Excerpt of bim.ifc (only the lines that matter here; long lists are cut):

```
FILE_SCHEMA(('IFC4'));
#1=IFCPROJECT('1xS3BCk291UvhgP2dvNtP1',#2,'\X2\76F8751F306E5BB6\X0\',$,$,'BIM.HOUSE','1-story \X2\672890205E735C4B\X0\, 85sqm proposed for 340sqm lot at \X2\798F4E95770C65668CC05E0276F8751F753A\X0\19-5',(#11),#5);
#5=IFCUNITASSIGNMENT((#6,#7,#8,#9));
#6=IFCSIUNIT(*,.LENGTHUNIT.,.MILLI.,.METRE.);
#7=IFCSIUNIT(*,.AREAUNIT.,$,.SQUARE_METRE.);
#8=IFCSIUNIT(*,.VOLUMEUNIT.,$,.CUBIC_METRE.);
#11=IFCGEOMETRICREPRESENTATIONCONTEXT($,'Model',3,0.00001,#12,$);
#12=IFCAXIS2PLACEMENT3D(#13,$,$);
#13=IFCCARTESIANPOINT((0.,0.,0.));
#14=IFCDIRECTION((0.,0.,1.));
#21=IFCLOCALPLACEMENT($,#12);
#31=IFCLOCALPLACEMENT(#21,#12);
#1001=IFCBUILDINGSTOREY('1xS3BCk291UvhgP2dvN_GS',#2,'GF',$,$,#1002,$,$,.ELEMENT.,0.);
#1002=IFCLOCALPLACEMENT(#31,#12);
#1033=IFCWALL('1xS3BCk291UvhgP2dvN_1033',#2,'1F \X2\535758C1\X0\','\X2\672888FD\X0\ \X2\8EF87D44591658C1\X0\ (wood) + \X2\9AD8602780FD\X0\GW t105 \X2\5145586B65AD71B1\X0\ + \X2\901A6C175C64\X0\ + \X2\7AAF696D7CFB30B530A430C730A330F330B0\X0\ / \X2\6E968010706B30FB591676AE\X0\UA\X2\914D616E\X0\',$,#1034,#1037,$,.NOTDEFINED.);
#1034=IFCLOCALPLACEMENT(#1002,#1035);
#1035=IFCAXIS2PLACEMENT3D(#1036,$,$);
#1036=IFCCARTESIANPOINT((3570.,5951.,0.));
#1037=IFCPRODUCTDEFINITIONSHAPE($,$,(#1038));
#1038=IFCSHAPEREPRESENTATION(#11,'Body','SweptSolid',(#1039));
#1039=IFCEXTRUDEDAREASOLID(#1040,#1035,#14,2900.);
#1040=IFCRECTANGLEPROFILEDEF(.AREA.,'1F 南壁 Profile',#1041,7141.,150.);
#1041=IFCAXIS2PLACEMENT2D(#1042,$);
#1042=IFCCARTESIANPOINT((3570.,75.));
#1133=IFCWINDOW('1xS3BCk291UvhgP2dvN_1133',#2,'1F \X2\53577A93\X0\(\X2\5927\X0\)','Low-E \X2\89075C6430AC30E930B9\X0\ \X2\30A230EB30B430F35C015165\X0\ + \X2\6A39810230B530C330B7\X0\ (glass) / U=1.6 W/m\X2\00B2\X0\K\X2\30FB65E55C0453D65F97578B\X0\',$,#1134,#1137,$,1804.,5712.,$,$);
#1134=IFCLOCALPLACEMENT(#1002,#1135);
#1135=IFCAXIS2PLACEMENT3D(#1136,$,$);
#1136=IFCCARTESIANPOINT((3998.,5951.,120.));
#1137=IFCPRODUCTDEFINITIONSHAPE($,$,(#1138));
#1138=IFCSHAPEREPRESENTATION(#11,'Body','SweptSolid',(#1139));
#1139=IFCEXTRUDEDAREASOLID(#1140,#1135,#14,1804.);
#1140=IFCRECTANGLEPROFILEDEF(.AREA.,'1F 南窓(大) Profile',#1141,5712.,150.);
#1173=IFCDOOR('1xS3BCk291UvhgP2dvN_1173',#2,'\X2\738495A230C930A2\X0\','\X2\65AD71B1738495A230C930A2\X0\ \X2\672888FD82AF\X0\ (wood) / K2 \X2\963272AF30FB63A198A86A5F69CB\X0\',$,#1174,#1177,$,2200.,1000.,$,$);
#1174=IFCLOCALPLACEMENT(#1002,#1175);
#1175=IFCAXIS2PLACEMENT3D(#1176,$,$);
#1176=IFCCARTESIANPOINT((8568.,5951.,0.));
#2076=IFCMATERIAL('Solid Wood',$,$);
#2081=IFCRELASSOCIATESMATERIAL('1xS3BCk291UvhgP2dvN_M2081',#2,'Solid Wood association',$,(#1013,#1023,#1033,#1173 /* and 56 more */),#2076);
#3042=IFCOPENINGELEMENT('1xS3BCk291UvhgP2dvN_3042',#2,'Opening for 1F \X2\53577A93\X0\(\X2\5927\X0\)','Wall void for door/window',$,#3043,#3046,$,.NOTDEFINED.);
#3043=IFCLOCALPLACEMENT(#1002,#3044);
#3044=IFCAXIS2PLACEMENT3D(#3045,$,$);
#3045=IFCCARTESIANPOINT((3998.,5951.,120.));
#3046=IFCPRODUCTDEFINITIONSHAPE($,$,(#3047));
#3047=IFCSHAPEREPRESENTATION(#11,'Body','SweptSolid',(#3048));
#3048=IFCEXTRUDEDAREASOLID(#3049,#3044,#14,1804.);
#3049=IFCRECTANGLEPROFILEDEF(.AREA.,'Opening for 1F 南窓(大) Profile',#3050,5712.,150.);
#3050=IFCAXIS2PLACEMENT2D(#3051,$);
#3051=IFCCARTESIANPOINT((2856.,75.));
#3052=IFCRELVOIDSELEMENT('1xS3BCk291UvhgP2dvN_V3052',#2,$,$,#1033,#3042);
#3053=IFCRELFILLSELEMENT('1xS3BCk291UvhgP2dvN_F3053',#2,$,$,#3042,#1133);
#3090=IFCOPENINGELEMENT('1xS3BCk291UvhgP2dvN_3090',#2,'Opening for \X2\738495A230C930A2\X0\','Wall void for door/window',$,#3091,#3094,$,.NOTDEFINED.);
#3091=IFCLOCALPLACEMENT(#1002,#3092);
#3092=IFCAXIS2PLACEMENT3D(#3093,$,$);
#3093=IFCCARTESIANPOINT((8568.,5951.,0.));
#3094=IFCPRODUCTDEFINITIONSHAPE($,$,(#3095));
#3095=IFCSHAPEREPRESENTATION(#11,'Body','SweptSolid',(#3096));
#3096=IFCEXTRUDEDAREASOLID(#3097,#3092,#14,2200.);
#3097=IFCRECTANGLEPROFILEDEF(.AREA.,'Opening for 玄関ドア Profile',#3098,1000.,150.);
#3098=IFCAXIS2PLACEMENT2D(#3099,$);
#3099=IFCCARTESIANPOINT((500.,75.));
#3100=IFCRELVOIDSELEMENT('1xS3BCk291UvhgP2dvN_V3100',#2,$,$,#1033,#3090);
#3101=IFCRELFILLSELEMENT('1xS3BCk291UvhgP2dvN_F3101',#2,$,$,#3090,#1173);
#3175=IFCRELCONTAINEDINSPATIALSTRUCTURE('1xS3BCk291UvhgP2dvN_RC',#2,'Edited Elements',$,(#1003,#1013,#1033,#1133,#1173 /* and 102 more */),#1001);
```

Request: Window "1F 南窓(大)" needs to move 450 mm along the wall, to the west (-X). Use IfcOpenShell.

```python
import ifcopenshell
import ifcopenshell.api.geometry
import ifcopenshell.util.placement
import ifcopenshell.util.unit

model = ifcopenshell.open("bim.ifc")
unit_scale = ifcopenshell.util.unit.calculate_unit_scale(model)

window = model.by_guid("1xS3BCk291UvhgP2dvN_1133")
opening = window.FillsVoids[0].RelatingOpeningElement
wall = opening.VoidsElements[0].RelatingBuildingElement

wall_matrix = ifcopenshell.util.placement.get_local_placement(wall.ObjectPlacement)
shift = wall_matrix[:3, 0] * -0.45 / unit_scale
before = ifcopenshell.util.placement.get_local_placement(window.ObjectPlacement)[:3, 3].copy()

# The window is not placed relative to its opening, so move both.
for product in (opening, window):
    matrix = ifcopenshell.util.placement.get_local_placement(product.ObjectPlacement)
    matrix[:3, 3] += shift
    ifcopenshell.api.geometry.edit_object_placement(model, product=product, matrix=matrix, is_si=False)

after = ifcopenshell.util.placement.get_local_placement(window.ObjectPlacement)[:3, 3]
print("window moved by", (after - before).round(3) + 0.0)

model.write("bim_rev.ifc")
```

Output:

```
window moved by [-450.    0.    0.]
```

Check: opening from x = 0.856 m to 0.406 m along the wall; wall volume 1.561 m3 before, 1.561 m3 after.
